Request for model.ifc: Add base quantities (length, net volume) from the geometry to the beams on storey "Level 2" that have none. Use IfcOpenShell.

First a look at what the model holds.

```python
import ifcopenshell
import ifcopenshell.util.element
import ifcopenshell.util.unit

model = ifcopenshell.open("model.ifc")
print(model.schema)
for unit_type in ("LENGTHUNIT", "AREAUNIT", "VOLUMEUNIT"):
    print(unit_type, ifcopenshell.util.unit.calculate_unit_scale(model, unit_type))
storey = next(s for s in model.by_type("IfcBuildingStorey") if s.Name == "Level 2")
beams = [e for e in ifcopenshell.util.element.get_decomposition(storey) if e.is_a("IfcBeam")]
for e in sorted(beams, key=lambda e: e.id()):
    print(e.id(), e.is_a(), e.Name, list(ifcopenshell.util.element.get_psets(e, qtos_only=True)), sep=" | ")
```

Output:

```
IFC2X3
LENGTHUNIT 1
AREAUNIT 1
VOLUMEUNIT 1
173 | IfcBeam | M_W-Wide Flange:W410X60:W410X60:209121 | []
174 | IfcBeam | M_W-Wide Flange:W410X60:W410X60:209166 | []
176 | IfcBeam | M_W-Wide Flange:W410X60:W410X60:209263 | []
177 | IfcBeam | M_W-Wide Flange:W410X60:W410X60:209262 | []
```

```python
import ifcopenshell
import ifcopenshell.api.pset
import ifcopenshell.geom
import ifcopenshell.util.element
import ifcopenshell.util.shape
import ifcopenshell.util.unit

model = ifcopenshell.open("model.ifc")
unit_scale = ifcopenshell.util.unit.calculate_unit_scale(model)
volume_scale = ifcopenshell.util.unit.calculate_unit_scale(model, "VOLUMEUNIT")
settings = ifcopenshell.geom.settings()

storey = next(s for s in model.by_type("IfcBuildingStorey") if s.Name == "Level 2")
beams = [e for e in ifcopenshell.util.element.get_decomposition(storey) if e.is_a("IfcBeam")]

for e in sorted(beams, key=lambda e: e.id()):
    if ifcopenshell.util.element.get_psets(e, qtos_only=True, should_inherit=False):
        continue
    # Geometry comes back in metres, in the element's own axes.
    shape = ifcopenshell.geom.create_shape(settings, e)
    values = {
        "Length": ifcopenshell.util.shape.get_max_xyz(shape.geometry) / unit_scale,
        "NetVolume": ifcopenshell.util.shape.get_volume(shape.geometry) / volume_scale,
    }
    qto = ifcopenshell.api.pset.add_qto(model, product=e, name="BaseQuantities")
    ifcopenshell.api.pset.edit_qto(model, qto=qto, properties=values)
    print(e.id(), {k: round(v, 3) for k, v in values.items()})

model.write("model-out.ifc")
```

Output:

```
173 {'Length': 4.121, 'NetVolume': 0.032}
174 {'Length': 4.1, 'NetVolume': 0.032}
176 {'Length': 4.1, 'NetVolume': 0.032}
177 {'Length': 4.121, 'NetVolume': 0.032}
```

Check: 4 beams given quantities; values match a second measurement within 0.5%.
